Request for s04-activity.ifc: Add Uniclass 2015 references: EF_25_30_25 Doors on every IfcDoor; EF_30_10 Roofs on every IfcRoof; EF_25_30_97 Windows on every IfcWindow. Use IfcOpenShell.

First a look at what the model holds.

```python
import ifcopenshell

model = ifcopenshell.open("s04-activity.ifc")
print(model.schema)
print("classifications:", [c.Name for c in model.by_type("IfcClassification")])
for ifc_class in ("IfcDoor", "IfcRoof", "IfcStair", "IfcWall", "IfcWindow"):
    print(ifc_class, len(model.by_type(ifc_class)))
```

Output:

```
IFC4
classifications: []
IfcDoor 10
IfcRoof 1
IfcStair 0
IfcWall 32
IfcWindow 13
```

```python
import ifcopenshell
import ifcopenshell.api.classification

model = ifcopenshell.open("s04-activity.ifc")

system = ifcopenshell.api.classification.add_classification(model, classification="Uniclass 2015")

codes = {
    "IfcDoor": ("EF_25_30_25", "Doors"),
    "IfcRoof": ("EF_30_10", "Roofs"),
    "IfcWindow": ("EF_25_30_97", "Windows"),
}
for ifc_class, (code, name) in codes.items():
    products = model.by_type(ifc_class)
    ifcopenshell.api.classification.add_reference(
        model, products=products, classification=system, identification=code, name=name
    )
    print(code, len(products))

model.write("s04-activity_rev.ifc")
```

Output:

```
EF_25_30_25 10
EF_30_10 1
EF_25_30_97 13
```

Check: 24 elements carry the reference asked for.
